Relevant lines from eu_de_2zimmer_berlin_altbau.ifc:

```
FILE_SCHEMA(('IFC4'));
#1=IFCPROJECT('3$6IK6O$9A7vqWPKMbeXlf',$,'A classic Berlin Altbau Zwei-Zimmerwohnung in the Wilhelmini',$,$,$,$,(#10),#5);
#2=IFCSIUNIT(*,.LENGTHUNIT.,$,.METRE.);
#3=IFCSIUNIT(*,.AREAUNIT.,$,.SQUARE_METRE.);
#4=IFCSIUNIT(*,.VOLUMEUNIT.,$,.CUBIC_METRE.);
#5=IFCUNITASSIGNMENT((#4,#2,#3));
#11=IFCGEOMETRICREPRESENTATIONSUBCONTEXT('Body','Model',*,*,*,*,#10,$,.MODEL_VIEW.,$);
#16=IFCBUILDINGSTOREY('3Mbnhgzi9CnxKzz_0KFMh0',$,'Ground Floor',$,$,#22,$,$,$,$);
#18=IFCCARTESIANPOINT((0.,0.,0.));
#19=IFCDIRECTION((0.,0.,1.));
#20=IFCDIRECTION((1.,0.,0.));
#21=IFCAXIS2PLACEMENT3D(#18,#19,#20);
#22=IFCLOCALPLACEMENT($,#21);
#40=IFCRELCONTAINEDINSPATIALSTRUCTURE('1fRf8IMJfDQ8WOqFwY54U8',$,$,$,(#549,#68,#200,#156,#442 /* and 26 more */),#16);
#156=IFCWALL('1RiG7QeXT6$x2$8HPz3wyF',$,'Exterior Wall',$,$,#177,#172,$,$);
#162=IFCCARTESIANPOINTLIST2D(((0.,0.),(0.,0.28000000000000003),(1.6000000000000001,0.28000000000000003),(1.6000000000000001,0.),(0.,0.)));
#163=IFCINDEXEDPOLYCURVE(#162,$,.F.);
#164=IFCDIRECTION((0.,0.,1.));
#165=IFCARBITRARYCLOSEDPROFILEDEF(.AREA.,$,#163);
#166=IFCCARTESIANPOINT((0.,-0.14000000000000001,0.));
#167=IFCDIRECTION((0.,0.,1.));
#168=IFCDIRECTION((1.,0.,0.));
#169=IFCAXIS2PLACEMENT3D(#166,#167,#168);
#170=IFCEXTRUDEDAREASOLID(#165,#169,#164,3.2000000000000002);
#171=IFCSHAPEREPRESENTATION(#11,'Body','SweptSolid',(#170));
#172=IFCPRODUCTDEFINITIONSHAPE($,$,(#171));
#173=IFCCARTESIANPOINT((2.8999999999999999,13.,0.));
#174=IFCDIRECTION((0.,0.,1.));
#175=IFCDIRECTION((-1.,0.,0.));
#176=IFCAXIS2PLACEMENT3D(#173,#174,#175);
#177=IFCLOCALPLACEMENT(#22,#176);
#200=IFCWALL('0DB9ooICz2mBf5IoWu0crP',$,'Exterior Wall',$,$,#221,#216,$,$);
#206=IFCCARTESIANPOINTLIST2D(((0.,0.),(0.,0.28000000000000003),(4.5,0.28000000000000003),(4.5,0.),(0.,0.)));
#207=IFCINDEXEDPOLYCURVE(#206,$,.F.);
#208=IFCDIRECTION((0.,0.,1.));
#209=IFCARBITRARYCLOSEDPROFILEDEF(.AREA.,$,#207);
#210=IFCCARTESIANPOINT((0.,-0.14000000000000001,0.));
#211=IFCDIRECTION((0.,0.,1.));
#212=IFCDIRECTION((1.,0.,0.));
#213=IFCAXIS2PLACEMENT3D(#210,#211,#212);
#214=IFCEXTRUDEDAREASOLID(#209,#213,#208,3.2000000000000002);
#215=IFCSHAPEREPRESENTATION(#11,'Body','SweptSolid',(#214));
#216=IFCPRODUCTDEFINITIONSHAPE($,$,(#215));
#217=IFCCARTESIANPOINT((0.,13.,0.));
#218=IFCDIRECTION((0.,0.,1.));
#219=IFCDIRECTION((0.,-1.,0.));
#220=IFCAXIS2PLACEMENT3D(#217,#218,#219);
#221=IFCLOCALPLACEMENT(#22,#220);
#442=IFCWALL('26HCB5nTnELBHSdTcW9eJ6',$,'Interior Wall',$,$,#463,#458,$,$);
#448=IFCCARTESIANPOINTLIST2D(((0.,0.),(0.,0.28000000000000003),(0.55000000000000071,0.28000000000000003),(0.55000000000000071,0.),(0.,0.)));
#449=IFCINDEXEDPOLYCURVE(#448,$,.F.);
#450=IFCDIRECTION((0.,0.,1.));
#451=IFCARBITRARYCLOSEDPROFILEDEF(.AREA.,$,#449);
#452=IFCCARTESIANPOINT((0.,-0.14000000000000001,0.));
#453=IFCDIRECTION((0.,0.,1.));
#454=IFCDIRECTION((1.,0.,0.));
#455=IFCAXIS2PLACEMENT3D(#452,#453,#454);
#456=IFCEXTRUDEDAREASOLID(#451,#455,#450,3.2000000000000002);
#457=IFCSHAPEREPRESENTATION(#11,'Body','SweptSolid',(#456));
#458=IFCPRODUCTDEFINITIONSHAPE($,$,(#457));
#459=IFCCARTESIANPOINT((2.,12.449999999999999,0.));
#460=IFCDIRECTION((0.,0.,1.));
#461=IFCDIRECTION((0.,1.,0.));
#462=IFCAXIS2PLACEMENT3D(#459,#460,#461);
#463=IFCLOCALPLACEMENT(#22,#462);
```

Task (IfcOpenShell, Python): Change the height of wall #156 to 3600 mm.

```python
import ifcopenshell
import ifcopenshell.geom
import ifcopenshell.util.representation
import ifcopenshell.util.shape
import ifcopenshell.util.unit

model = ifcopenshell.open("eu_de_2zimmer_berlin_altbau.ifc")
unit_scale = ifcopenshell.util.unit.calculate_unit_scale(model)
settings = ifcopenshell.geom.settings()


def volume(element):
    """Net volume in cubic metres, openings subtracted."""
    shape = ifcopenshell.geom.create_shape(settings, element)
    return ifcopenshell.util.shape.get_volume(shape.geometry)


wall = model.by_guid("1RiG7QeXT6$x2$8HPz3wyF")
before = volume(wall)

body = ifcopenshell.util.representation.get_representation(wall, "Model", "Body")
solid = body.Items[0]
old_height = solid.Depth
solid.Depth = 3.6 / unit_scale
after = volume(wall)

print(f"height {old_height:g} -> {solid.Depth:g}, volume {before:.3f} -> {after:.3f} m3")

model.write("eu_de_2zimmer_berlin_altbau_edited.ifc")
```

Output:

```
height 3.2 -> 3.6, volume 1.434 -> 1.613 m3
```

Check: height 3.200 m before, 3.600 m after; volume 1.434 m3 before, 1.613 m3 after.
